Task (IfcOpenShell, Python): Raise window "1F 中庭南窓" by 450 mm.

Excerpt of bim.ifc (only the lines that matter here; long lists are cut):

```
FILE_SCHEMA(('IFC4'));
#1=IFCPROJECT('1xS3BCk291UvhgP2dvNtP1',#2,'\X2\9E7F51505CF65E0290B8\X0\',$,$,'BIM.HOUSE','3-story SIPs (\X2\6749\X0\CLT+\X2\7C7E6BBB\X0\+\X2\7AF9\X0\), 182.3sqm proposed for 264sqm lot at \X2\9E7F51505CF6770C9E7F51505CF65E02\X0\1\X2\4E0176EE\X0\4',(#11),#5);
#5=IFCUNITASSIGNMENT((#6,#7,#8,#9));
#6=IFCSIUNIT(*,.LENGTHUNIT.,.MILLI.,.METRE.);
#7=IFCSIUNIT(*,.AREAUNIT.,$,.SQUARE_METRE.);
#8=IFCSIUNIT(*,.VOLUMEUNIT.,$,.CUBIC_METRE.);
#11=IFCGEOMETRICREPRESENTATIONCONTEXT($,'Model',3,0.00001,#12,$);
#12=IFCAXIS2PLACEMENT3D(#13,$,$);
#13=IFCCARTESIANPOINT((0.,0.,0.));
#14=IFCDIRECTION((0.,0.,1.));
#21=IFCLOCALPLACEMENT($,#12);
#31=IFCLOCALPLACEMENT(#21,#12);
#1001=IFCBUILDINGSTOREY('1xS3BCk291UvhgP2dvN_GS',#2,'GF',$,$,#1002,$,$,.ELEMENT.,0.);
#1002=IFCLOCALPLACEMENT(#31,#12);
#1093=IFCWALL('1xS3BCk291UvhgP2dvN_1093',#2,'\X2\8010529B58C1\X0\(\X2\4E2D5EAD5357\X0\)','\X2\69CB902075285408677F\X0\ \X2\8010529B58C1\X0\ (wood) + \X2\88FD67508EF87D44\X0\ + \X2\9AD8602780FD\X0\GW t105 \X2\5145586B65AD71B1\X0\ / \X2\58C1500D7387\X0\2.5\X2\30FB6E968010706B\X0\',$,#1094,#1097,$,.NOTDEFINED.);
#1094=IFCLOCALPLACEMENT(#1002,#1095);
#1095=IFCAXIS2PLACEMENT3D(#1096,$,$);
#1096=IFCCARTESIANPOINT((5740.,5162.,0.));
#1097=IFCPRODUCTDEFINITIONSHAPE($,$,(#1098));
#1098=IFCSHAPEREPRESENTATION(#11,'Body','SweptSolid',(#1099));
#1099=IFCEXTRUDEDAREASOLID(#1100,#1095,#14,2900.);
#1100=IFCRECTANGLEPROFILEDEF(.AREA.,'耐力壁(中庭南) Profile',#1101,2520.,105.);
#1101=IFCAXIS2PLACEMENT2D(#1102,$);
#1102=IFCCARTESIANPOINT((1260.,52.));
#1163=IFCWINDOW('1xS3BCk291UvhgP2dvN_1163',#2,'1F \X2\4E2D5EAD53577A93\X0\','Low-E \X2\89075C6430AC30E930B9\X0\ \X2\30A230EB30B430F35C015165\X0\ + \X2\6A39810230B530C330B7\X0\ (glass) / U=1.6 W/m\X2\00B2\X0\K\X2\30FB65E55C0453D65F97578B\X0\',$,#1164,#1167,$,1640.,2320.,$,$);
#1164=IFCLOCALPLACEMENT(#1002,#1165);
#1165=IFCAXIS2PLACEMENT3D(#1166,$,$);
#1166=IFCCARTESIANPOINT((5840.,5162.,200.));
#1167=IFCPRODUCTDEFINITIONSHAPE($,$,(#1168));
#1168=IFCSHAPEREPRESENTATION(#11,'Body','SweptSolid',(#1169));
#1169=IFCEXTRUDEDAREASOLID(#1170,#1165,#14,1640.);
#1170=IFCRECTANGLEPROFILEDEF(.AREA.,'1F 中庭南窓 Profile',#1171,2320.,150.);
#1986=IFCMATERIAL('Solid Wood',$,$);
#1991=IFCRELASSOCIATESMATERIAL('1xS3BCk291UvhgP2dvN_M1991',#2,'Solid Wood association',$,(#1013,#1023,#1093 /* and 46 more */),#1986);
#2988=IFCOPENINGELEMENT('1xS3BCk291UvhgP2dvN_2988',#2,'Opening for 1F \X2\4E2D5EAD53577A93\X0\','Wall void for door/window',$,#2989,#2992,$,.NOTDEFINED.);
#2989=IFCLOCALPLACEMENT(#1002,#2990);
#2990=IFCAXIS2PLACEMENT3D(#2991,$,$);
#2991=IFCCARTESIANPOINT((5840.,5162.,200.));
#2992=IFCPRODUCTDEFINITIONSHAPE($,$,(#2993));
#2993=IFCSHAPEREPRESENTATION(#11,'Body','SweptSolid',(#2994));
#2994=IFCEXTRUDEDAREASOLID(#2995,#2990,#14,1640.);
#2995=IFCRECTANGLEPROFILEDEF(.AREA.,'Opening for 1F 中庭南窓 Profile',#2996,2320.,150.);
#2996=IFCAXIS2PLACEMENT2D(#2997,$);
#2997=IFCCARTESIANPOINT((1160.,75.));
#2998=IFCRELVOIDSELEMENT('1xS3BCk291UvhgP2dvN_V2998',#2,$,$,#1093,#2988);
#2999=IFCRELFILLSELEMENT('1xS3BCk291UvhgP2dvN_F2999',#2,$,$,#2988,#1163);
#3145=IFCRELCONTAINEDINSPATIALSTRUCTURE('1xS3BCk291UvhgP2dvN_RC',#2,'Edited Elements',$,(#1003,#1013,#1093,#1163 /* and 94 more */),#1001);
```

```python
import numpy as np
import ifcopenshell
import ifcopenshell.api.geometry
import ifcopenshell.util.placement
import ifcopenshell.util.unit

model = ifcopenshell.open("bim.ifc")
unit_scale = ifcopenshell.util.unit.calculate_unit_scale(model)

window = model.by_id(1163)
opening = window.FillsVoids[0].RelatingOpeningElement
dz = 0.45 / unit_scale

shift = np.array([0.0, 0.0, dz])
# The window is not placed relative to its opening, so move both.
for product in (opening, window):
    matrix = ifcopenshell.util.placement.get_local_placement(product.ObjectPlacement)
    matrix[:3, 3] += shift
    ifcopenshell.api.geometry.edit_object_placement(model, product=product, matrix=matrix, is_si=False)

print(f"moved by {dz * unit_scale:+.3f} m")

model.write("bim-out.ifc")
```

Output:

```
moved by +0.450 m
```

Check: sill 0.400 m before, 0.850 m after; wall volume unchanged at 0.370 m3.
